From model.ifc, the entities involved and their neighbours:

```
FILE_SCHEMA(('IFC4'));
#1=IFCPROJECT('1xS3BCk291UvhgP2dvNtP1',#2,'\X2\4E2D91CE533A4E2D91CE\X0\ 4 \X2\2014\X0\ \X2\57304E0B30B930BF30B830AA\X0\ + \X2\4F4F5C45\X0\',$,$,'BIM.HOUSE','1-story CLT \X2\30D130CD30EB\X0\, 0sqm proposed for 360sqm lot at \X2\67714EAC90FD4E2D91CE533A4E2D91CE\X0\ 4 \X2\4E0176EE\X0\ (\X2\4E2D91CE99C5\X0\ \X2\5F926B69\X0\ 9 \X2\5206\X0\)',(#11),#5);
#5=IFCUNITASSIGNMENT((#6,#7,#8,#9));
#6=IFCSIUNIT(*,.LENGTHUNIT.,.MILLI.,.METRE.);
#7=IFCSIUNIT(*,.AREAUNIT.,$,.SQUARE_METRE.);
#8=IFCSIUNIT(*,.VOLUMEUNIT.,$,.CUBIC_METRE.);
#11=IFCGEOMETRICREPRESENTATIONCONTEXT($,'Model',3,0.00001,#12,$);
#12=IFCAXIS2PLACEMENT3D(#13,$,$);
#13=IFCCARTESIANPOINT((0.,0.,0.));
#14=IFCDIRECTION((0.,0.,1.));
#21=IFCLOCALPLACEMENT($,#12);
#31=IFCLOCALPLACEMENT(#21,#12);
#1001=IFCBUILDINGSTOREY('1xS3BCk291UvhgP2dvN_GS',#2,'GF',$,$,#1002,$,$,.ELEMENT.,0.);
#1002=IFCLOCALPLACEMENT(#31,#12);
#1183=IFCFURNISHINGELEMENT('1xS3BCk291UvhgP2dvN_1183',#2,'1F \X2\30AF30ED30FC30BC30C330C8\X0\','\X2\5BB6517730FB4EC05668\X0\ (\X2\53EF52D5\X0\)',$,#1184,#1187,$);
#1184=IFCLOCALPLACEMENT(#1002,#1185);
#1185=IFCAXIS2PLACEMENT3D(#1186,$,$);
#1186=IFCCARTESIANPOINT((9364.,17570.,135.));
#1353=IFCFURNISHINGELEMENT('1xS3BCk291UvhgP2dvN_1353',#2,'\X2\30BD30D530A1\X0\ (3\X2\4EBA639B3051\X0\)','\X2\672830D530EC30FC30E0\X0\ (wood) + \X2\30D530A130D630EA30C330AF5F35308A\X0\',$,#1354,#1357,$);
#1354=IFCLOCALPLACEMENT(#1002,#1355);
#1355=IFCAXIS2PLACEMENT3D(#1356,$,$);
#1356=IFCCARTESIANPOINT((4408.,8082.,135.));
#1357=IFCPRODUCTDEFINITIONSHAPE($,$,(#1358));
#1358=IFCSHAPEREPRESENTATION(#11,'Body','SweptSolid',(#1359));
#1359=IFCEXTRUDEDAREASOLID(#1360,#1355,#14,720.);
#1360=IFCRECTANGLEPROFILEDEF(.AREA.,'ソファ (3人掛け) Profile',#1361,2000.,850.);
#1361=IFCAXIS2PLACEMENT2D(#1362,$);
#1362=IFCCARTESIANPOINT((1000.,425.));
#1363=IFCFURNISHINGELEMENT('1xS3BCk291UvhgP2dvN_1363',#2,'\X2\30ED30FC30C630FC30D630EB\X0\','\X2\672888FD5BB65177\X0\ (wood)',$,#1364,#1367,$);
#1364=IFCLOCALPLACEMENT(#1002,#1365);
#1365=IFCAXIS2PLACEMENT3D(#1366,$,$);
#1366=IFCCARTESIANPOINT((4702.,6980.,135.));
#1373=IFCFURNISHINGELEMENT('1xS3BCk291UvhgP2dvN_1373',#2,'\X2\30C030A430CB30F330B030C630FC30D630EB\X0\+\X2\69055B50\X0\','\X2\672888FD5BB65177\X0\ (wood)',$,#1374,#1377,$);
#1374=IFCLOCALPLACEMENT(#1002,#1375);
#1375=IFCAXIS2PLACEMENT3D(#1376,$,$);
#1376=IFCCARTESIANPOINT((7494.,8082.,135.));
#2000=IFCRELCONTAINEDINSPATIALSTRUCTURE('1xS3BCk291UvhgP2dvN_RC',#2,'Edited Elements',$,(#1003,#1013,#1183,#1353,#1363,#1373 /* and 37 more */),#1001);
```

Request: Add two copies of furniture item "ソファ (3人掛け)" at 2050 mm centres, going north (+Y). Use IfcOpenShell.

```python
import numpy as np
import ifcopenshell
import ifcopenshell.api.geometry
import ifcopenshell.api.root
import ifcopenshell.util.element
import ifcopenshell.util.placement
import ifcopenshell.util.unit

model = ifcopenshell.open("model.ifc")
unit_scale = ifcopenshell.util.unit.calculate_unit_scale(model)


def reuse_history(source, copy):
    """copy_class also copies each property set's owner history, people and application; keep the originals."""
    for rel in copy.IsDefinedBy:
        if rel.is_a("IfcRelDefinesByProperties") and (history := rel.RelatingPropertyDefinition.OwnerHistory):
            rel.RelatingPropertyDefinition.OwnerHistory = source.OwnerHistory
            ifcopenshell.util.element.remove_deep2(model, history)


source = model.by_guid("1xS3BCk291UvhgP2dvN_1353")
base = ifcopenshell.util.placement.get_local_placement(source.ObjectPlacement)
step = np.array([0.0, 1.0, 0.0]) * 2.05 / unit_scale

for i in range(1, 3):
    copy = ifcopenshell.api.root.copy_class(model, product=source)
    copy.Representation = ifcopenshell.util.element.copy_deep(
        model, source.Representation, exclude=["IfcGeometricRepresentationContext", "IfcRepresentationMap"]
    )
    reuse_history(source, copy)
    matrix = base.copy()
    matrix[:3, 3] += i * step
    print("added at", matrix[:3, 3].round(3) + 0.0)
    ifcopenshell.api.geometry.edit_object_placement(model, product=copy, matrix=matrix, is_si=False)

model.write("model_updated.ifc")
```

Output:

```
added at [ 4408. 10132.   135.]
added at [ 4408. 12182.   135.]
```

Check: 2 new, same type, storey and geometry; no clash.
